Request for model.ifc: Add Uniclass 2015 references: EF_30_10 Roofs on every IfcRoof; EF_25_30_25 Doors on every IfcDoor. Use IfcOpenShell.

First a look at what the model holds.

```python
import ifcopenshell

model = ifcopenshell.open("model.ifc")
print(model.schema)
print("classifications:", [c.Name for c in model.by_type("IfcClassification")])
for ifc_class in ("IfcDoor", "IfcRoof", "IfcStair", "IfcWall", "IfcWindow"):
    print(ifc_class, len(model.by_type(ifc_class)))
```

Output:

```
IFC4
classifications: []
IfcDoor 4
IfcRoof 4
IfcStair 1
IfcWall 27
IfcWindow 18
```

```python
import ifcopenshell
import ifcopenshell.api.classification

model = ifcopenshell.open("model.ifc")

system = ifcopenshell.api.classification.add_classification(model, classification="Uniclass 2015")

codes = {
    "IfcRoof": ("EF_30_10", "Roofs"),
    "IfcDoor": ("EF_25_30_25", "Doors"),
}
for ifc_class, (code, name) in codes.items():
    products = model.by_type(ifc_class)
    ifcopenshell.api.classification.add_reference(
        model, products=products, classification=system, identification=code, name=name
    )
    print(code, len(products))

model.write("model_v2.ifc")
```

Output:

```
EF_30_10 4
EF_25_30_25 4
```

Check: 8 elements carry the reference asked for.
